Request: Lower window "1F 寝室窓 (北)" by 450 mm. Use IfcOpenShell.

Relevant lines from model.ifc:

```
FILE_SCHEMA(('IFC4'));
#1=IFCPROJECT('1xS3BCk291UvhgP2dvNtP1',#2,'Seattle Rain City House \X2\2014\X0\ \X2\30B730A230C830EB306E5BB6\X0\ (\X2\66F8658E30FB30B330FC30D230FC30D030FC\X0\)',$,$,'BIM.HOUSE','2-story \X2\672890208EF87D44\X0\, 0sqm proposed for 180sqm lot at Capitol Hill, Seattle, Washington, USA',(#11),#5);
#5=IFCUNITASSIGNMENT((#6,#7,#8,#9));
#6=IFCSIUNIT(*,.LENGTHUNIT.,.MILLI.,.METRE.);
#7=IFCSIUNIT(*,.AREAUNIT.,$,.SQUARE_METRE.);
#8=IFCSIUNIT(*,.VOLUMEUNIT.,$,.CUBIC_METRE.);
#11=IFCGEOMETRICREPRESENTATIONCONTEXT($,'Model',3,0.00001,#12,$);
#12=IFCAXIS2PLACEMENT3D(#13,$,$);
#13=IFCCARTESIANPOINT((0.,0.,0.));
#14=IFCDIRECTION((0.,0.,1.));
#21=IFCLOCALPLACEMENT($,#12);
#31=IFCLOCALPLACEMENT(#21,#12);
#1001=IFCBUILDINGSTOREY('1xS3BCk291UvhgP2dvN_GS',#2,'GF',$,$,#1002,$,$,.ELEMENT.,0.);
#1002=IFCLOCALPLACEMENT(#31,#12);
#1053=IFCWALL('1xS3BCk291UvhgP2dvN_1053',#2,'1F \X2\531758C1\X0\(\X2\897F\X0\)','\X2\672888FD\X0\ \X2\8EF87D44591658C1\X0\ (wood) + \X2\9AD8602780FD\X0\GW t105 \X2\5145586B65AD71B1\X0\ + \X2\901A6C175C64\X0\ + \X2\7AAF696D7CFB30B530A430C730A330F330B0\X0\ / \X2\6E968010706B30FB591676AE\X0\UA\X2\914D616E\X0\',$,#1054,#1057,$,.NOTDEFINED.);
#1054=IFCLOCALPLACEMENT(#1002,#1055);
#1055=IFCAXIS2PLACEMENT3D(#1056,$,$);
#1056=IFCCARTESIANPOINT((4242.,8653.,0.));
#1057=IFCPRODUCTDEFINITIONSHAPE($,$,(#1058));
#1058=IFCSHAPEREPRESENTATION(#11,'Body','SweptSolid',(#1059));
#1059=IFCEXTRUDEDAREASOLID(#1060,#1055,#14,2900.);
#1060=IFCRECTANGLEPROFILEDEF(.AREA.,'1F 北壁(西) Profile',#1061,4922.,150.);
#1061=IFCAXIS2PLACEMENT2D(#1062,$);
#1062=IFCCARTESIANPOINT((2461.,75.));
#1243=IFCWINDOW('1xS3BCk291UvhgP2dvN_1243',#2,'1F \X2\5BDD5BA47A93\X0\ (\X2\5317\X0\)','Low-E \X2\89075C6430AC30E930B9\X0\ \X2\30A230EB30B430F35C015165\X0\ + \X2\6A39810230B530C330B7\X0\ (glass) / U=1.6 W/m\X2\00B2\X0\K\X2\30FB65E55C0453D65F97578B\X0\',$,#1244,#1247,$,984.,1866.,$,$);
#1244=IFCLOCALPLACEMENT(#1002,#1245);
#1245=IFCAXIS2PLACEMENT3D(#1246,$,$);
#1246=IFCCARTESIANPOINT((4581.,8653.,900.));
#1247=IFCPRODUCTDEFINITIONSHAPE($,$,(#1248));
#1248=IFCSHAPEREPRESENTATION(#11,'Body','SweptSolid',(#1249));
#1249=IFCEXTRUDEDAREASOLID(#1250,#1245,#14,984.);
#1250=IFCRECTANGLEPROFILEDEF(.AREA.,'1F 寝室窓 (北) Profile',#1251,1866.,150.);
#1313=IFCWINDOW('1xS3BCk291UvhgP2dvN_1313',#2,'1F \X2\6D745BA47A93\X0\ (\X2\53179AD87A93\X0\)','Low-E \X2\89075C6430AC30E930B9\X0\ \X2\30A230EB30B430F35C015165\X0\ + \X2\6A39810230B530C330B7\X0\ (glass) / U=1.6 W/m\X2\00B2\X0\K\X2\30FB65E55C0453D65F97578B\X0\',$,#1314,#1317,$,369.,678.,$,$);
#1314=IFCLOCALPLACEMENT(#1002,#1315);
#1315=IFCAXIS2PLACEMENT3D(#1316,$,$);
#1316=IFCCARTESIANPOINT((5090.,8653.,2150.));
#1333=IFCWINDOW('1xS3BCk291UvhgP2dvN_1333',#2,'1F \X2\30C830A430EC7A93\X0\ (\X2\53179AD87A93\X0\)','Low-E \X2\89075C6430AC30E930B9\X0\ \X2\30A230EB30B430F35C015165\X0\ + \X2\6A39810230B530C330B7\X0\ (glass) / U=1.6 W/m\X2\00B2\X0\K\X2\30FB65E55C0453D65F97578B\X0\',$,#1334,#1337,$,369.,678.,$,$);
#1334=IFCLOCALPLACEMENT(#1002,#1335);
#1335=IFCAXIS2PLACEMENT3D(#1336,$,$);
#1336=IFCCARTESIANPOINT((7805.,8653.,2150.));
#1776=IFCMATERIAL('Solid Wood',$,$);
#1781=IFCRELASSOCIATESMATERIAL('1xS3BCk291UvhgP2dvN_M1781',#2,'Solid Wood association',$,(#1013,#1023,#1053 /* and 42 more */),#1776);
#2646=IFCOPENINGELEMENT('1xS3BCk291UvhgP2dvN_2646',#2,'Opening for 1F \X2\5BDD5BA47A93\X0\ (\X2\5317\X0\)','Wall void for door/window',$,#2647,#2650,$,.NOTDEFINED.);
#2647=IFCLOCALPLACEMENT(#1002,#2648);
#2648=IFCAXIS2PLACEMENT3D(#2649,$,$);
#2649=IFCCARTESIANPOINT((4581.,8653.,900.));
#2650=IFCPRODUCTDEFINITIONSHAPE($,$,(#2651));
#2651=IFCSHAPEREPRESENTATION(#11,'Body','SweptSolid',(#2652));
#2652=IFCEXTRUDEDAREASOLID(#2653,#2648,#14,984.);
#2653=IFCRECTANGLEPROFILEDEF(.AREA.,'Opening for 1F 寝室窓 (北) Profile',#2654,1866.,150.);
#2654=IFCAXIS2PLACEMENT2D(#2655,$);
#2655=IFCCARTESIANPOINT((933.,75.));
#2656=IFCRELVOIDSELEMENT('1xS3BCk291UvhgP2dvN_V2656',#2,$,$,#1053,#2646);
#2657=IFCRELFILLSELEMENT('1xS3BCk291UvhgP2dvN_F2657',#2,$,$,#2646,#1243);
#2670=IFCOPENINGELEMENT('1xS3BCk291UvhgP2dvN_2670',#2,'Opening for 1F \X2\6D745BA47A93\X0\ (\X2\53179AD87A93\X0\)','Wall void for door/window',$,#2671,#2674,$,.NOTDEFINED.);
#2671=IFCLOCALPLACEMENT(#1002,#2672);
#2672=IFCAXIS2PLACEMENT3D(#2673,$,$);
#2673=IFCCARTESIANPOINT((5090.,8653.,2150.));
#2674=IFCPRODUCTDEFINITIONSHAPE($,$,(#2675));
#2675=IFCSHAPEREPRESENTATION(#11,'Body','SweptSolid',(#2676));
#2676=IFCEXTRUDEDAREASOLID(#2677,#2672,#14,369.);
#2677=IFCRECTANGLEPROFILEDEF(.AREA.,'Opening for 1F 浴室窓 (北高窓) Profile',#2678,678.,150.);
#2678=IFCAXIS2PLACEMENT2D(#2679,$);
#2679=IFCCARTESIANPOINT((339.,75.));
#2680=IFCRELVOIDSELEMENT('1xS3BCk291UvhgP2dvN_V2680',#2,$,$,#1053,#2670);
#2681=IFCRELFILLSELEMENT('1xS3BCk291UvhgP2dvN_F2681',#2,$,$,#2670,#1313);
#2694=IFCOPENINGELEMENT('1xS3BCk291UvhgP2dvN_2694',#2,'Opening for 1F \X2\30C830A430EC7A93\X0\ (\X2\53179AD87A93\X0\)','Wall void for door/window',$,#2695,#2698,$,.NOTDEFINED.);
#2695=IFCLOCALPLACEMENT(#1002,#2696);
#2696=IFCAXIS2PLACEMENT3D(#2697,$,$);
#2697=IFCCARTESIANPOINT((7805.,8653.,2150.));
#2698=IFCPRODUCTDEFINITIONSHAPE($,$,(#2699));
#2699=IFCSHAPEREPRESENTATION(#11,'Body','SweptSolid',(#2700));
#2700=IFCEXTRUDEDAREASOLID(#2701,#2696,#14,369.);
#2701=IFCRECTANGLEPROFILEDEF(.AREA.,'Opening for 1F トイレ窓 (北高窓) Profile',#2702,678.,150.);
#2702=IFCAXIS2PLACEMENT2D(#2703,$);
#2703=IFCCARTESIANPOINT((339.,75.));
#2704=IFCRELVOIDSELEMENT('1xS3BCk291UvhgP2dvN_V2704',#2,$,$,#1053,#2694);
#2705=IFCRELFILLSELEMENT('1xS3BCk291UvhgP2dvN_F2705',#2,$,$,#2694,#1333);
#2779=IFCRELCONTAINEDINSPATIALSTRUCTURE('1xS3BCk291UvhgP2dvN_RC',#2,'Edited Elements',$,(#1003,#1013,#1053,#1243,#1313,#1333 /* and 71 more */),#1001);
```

```python
import numpy as np
import ifcopenshell
import ifcopenshell.api.geometry
import ifcopenshell.util.placement
import ifcopenshell.util.unit

model = ifcopenshell.open("model.ifc")
unit_scale = ifcopenshell.util.unit.calculate_unit_scale(model)

window = model.by_guid("1xS3BCk291UvhgP2dvN_1243")
opening = window.FillsVoids[0].RelatingOpeningElement
dz = -450.0

shift = np.array([0.0, 0.0, dz])
# The window is not placed relative to its opening, so move both.
for product in (opening, window):
    matrix = ifcopenshell.util.placement.get_local_placement(product.ObjectPlacement)
    matrix[:3, 3] += shift
    ifcopenshell.api.geometry.edit_object_placement(model, product=product, matrix=matrix, is_si=False)

print(f"moved by {dz * unit_scale:+.3f} m")

model.write("model_rev.ifc")
```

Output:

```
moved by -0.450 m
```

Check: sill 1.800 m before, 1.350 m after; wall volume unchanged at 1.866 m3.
